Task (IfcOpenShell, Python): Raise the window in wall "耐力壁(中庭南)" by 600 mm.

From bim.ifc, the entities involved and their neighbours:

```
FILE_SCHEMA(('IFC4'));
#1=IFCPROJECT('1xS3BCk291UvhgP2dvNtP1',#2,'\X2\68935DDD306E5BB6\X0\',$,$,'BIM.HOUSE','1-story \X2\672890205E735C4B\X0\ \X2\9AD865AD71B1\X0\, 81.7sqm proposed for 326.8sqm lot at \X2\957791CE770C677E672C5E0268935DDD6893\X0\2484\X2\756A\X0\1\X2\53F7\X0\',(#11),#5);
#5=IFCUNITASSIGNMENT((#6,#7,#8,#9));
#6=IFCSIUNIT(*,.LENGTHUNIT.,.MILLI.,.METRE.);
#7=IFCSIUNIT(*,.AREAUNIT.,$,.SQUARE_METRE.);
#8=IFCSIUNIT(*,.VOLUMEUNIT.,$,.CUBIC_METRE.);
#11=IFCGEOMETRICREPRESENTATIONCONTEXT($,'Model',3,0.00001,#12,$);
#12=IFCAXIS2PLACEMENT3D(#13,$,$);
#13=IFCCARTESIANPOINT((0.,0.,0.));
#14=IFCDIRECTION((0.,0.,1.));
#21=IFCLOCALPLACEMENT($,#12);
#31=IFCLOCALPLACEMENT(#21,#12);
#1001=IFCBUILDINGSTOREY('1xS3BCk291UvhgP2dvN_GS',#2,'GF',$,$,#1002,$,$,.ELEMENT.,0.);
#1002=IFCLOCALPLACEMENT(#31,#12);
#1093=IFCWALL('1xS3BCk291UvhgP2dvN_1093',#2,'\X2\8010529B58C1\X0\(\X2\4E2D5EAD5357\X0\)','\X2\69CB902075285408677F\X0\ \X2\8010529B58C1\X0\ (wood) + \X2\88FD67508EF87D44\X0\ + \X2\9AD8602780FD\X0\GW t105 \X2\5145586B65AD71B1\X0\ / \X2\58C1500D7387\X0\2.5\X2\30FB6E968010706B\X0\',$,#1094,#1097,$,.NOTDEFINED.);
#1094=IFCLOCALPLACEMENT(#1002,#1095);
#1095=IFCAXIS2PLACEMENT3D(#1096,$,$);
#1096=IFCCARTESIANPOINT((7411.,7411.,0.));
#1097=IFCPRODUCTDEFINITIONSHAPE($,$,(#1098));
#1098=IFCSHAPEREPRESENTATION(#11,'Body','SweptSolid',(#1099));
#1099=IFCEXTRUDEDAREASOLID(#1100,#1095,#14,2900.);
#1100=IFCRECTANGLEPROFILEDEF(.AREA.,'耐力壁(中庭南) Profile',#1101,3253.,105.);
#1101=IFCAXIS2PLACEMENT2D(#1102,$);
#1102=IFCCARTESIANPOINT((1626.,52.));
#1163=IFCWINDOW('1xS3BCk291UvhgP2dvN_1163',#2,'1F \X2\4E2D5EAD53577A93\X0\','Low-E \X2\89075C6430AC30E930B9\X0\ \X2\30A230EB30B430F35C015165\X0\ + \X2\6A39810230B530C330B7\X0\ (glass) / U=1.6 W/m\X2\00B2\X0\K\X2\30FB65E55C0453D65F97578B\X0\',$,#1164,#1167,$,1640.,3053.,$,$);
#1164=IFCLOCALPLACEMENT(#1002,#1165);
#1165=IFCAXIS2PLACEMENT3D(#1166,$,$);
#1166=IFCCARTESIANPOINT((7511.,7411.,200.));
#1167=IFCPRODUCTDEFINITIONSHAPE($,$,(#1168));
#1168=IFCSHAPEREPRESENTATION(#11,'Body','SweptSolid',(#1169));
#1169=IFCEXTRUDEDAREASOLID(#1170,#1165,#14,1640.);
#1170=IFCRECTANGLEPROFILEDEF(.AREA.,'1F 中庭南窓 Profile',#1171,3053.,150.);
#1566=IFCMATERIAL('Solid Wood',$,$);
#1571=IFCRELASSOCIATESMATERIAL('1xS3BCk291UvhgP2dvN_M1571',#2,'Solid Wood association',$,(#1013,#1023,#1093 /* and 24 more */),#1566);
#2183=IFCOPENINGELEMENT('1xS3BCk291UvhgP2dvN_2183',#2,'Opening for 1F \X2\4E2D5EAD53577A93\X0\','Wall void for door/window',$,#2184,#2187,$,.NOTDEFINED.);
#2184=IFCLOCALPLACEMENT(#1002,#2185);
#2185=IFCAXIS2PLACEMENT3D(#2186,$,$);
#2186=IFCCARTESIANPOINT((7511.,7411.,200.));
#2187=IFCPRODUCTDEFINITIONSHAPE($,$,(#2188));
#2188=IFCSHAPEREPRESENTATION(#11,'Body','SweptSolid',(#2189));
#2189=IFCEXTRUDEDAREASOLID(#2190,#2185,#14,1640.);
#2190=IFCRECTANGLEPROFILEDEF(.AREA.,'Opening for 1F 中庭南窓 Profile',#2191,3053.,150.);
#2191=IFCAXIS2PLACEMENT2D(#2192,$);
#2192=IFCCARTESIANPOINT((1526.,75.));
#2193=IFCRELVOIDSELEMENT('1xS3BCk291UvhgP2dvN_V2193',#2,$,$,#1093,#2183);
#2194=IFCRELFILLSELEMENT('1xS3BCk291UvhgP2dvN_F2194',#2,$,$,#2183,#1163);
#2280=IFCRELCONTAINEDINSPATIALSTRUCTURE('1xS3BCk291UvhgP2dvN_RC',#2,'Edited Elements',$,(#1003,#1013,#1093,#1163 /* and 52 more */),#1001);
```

```python
import numpy as np
import ifcopenshell
import ifcopenshell.api.geometry
import ifcopenshell.util.placement
import ifcopenshell.util.unit

model = ifcopenshell.open("bim.ifc")
unit_scale = ifcopenshell.util.unit.calculate_unit_scale(model)

window = model.by_id(1163)
opening = window.FillsVoids[0].RelatingOpeningElement
dz = 0.6 / unit_scale

shift = np.array([0.0, 0.0, dz])
# The window is not placed relative to its opening, so move both.
for product in (opening, window):
    matrix = ifcopenshell.util.placement.get_local_placement(product.ObjectPlacement)
    matrix[:3, 3] += shift
    ifcopenshell.api.geometry.edit_object_placement(model, product=product, matrix=matrix, is_si=False)

print(f"moved by {dz * unit_scale:+.3f} m")

model.write("bim_updated.ifc")
```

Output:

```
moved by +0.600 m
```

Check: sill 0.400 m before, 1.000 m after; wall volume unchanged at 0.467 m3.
